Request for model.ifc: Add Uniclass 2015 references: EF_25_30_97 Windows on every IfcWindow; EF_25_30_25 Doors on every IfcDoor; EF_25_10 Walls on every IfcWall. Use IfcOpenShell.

First a look at what the model holds.

```python
import ifcopenshell

model = ifcopenshell.open("model.ifc")
print(model.schema)
print("classifications:", [c.Name for c in model.by_type("IfcClassification")])
for ifc_class in ("IfcDoor", "IfcRoof", "IfcStair", "IfcWall", "IfcWindow"):
    print(ifc_class, len(model.by_type(ifc_class)))
```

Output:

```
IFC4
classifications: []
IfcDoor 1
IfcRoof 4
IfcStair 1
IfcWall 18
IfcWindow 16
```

```python
import ifcopenshell
import ifcopenshell.api.classification

model = ifcopenshell.open("model.ifc")

system = ifcopenshell.api.classification.add_classification(model, classification="Uniclass 2015")

codes = {
    "IfcWindow": ("EF_25_30_97", "Windows"),
    "IfcDoor": ("EF_25_30_25", "Doors"),
    "IfcWall": ("EF_25_10", "Walls"),
}
for ifc_class, (code, name) in codes.items():
    products = model.by_type(ifc_class)
    ifcopenshell.api.classification.add_reference(
        model, products=products, classification=system, identification=code, name=name
    )
    print(code, len(products))

model.write("model_updated.ifc")
```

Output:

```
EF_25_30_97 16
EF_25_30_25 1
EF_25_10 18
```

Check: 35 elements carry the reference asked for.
